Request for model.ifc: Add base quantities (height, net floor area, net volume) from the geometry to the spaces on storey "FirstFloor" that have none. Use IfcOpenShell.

First a look at what the model holds.

```python
import ifcopenshell
import ifcopenshell.util.element
import ifcopenshell.util.unit

model = ifcopenshell.open("model.ifc")
print(model.schema)
for unit_type in ("LENGTHUNIT", "AREAUNIT", "VOLUMEUNIT"):
    print(unit_type, ifcopenshell.util.unit.calculate_unit_scale(model, unit_type))
storey = next(s for s in model.by_type("IfcBuildingStorey") if s.Name == "FirstFloor")
spaces = [e for e in ifcopenshell.util.element.get_decomposition(storey) if e.is_a("IfcSpace")]
for e in sorted(spaces, key=lambda e: e.id()):
    print(e.id(), e.is_a(), e.Name, list(ifcopenshell.util.element.get_psets(e, qtos_only=True)), sep=" | ")
```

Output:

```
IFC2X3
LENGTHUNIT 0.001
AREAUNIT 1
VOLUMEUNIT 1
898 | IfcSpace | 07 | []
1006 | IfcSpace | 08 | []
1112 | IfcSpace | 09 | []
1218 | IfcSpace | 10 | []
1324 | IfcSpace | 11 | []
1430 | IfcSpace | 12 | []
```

```python
import ifcopenshell
import ifcopenshell.api.pset
import ifcopenshell.geom
import ifcopenshell.util.element
import ifcopenshell.util.shape
import ifcopenshell.util.unit

model = ifcopenshell.open("model.ifc")
unit_scale = ifcopenshell.util.unit.calculate_unit_scale(model)
area_scale = ifcopenshell.util.unit.calculate_unit_scale(model, "AREAUNIT")
volume_scale = ifcopenshell.util.unit.calculate_unit_scale(model, "VOLUMEUNIT")
settings = ifcopenshell.geom.settings()

storey = next(s for s in model.by_type("IfcBuildingStorey") if s.Name == "FirstFloor")
spaces = [e for e in ifcopenshell.util.element.get_decomposition(storey) if e.is_a("IfcSpace")]

for e in sorted(spaces, key=lambda e: e.id()):
    if ifcopenshell.util.element.get_psets(e, qtos_only=True, should_inherit=False):
        continue
    # Geometry comes back in metres, in the element's own axes.
    shape = ifcopenshell.geom.create_shape(settings, e)
    values = {
        "Height": ifcopenshell.util.shape.get_z(shape.geometry) / unit_scale,
        "NetFloorArea": ifcopenshell.util.shape.get_footprint_area(shape.geometry) / area_scale,
        "NetVolume": ifcopenshell.util.shape.get_volume(shape.geometry) / volume_scale,
    }
    qto = ifcopenshell.api.pset.add_qto(model, product=e, name="BaseQuantities")
    ifcopenshell.api.pset.edit_qto(model, qto=qto, properties=values)
    print(e.id(), {k: round(v, 3) for k, v in values.items()})

model.write("model-out.ifc")
```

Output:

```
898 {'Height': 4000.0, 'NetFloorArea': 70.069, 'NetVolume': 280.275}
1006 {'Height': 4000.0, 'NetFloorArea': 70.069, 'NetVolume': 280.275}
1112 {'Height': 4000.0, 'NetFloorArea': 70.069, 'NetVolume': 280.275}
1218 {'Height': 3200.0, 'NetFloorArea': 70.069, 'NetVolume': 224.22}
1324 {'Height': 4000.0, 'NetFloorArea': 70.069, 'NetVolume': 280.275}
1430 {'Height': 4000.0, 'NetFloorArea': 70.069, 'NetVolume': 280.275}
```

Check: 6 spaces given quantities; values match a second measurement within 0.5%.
